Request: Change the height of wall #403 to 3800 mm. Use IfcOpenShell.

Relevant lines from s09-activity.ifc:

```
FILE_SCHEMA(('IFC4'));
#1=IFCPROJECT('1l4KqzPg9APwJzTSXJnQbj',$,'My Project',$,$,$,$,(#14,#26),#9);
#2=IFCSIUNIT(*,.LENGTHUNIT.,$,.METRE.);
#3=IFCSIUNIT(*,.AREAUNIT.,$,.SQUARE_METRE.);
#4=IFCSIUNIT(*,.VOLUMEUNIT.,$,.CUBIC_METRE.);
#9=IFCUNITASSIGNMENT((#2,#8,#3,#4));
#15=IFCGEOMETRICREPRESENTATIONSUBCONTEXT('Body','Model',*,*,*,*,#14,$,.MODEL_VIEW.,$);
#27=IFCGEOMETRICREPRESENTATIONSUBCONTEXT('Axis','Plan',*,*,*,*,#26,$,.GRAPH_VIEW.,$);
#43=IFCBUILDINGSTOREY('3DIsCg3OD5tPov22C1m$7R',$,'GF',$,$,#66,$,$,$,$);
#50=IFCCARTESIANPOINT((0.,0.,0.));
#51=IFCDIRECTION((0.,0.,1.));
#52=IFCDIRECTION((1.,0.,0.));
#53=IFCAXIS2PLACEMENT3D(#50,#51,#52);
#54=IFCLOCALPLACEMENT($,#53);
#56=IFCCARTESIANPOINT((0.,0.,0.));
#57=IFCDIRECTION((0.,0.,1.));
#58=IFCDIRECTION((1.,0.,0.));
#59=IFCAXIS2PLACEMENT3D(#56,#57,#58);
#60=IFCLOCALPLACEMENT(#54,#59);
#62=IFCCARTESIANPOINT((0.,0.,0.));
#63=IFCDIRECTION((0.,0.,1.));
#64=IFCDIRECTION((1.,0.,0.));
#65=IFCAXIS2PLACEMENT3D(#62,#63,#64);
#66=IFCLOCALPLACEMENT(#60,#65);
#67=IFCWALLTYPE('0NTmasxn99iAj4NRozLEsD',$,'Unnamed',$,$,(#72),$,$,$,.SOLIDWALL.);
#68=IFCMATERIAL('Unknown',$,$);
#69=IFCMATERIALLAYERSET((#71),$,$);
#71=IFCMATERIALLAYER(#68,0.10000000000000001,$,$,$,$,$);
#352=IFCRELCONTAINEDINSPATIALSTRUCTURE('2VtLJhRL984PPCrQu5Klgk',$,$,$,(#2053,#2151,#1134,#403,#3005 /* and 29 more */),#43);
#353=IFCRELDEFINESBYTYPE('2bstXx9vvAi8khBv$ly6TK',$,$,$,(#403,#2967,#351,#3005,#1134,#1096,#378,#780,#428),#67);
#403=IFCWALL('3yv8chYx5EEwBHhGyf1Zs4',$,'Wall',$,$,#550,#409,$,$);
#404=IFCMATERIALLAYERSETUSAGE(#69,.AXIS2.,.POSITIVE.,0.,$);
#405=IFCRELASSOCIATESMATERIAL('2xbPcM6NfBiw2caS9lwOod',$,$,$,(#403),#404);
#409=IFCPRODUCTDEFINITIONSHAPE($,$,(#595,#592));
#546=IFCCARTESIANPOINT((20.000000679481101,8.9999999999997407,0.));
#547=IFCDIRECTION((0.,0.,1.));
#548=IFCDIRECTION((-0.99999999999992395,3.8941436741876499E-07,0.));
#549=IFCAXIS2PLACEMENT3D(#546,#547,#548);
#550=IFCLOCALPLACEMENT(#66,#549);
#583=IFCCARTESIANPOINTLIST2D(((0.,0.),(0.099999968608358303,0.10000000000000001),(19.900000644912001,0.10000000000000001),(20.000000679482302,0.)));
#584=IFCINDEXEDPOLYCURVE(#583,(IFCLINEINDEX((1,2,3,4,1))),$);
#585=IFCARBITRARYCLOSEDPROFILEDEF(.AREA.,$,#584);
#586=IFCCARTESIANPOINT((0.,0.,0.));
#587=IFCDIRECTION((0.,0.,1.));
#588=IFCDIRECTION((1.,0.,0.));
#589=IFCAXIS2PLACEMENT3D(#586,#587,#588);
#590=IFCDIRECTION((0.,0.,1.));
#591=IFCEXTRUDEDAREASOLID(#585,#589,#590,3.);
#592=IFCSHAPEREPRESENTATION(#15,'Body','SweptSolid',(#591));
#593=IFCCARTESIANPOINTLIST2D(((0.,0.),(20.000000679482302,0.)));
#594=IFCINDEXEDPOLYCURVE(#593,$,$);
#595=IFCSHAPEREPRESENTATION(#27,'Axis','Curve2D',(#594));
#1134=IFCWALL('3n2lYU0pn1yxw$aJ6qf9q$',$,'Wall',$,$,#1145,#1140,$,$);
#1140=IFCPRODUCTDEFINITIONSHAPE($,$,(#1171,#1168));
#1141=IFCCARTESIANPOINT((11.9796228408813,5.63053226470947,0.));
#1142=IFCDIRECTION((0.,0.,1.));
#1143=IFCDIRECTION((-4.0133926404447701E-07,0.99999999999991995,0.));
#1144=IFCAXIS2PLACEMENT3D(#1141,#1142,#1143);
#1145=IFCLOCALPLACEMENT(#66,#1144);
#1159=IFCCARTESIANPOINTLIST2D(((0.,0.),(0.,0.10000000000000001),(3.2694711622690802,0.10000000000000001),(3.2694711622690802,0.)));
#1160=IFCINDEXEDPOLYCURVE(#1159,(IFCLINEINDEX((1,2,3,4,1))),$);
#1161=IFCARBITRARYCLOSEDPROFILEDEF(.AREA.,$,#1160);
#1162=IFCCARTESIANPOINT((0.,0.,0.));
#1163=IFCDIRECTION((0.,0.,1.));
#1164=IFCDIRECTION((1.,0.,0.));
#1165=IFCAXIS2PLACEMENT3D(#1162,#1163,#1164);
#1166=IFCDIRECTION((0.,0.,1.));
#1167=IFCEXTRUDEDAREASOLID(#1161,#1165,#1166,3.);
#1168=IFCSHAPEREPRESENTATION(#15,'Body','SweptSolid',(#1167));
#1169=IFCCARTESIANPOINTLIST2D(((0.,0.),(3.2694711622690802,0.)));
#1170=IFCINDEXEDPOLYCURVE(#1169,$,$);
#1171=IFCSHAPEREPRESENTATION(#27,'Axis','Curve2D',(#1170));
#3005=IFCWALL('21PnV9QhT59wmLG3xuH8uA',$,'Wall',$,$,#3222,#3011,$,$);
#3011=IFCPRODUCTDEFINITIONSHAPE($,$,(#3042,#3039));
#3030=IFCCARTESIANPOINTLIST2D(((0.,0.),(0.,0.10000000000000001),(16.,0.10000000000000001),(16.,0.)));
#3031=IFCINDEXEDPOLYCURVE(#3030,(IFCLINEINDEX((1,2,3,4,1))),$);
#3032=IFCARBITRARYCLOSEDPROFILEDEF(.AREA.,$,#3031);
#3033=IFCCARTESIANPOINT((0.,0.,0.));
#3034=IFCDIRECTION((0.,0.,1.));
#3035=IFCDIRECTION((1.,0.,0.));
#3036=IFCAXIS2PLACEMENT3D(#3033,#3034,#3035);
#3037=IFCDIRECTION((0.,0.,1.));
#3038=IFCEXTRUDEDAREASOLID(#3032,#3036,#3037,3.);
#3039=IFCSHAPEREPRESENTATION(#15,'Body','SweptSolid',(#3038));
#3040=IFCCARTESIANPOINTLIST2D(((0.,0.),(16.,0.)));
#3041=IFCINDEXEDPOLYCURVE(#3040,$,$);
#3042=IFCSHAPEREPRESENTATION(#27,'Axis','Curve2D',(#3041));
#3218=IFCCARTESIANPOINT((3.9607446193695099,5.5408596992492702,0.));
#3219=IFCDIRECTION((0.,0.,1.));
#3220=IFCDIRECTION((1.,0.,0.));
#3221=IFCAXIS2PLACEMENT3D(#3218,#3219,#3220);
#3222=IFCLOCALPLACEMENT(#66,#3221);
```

```python
import ifcopenshell
import ifcopenshell.geom
import ifcopenshell.util.representation
import ifcopenshell.util.shape

model = ifcopenshell.open("s09-activity.ifc")
settings = ifcopenshell.geom.settings()


def volume(element):
    """Net volume in cubic metres, openings subtracted."""
    shape = ifcopenshell.geom.create_shape(settings, element)
    return ifcopenshell.util.shape.get_volume(shape.geometry)


wall = model.by_id(403)
before = volume(wall)

body = ifcopenshell.util.representation.get_representation(wall, "Model", "Body")
solid = body.Items[0]
old_height = solid.Depth
solid.Depth = 3.8
after = volume(wall)

print(f"height {old_height:g} -> {solid.Depth:g}, volume {before:.3f} -> {after:.3f} m3")

model.write("s09-activity-out.ifc")
```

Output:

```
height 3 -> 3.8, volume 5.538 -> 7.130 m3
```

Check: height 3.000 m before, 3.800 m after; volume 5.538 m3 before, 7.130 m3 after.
